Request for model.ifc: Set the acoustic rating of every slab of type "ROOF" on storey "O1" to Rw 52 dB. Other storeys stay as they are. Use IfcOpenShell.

First a look at what the model holds.

```python
import ifcopenshell
import ifcopenshell.util.element

model = ifcopenshell.open("model.ifc")
print(model.schema)
storey = next(s for s in model.by_type("IfcBuildingStorey") if s.Name == "O1")
slabs = [e for e in ifcopenshell.util.element.get_decomposition(storey) if e.is_a("IfcSlab")]
seen = {}
for e in slabs:
    element_type = ifcopenshell.util.element.get_type(e)
    key = (element_type.Name if element_type != e and element_type else None, ifcopenshell.util.element.get_pset(e, "Pset_SlabCommon", "AcousticRating"))
    seen[key] = seen.get(key, 0) + 1
for (name, value), count in sorted(seen.items(), key=str):
    print(count, "x", name, "|", value)
```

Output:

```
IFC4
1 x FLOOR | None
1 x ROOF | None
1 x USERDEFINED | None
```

```python
import ifcopenshell
import ifcopenshell.api.pset
import ifcopenshell.util.element

model = ifcopenshell.open("model.ifc")

storey = next(s for s in model.by_type("IfcBuildingStorey") if s.Name == "O1")
slabs = [e for e in ifcopenshell.util.element.get_decomposition(storey) if e.is_a("IfcSlab")]

count = 0
for e in slabs:
    element_type = ifcopenshell.util.element.get_type(e)
    if element_type in (None, e) or element_type.Name != "ROOF":
        continue
    # add_pset returns the element's existing set when there is one.
    pset = ifcopenshell.api.pset.add_pset(model, product=e, name="Pset_SlabCommon")
    ifcopenshell.api.pset.edit_pset(model, pset=pset, properties={"AcousticRating": "Rw 52 dB"})
    count += 1

print(count, "slabs updated")

model.write("model_updated.ifc")
```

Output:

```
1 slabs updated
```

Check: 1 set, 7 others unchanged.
